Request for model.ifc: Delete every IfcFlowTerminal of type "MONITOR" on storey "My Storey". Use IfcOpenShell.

First a look at what the model holds.

```python
import ifcopenshell
import ifcopenshell.util.element

model = ifcopenshell.open("model.ifc")
print(model.schema)
storey = next(s for s in model.by_type("IfcBuildingStorey") if s.Name == "My Storey")
terminals = [e for e in ifcopenshell.util.element.get_decomposition(storey) if e.is_a("IfcFlowTerminal")]
seen = {}
for e in terminals:
    element_type = ifcopenshell.util.element.get_type(e)
    name = element_type.Name if element_type not in (None, e) else None
    seen[name] = seen.get(name, 0) + 1
for name, count in sorted(seen.items(), key=str):
    print(count, "x", name)
```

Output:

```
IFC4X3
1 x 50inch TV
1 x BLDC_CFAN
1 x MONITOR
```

```python
import ifcopenshell
import ifcopenshell.api.root
import ifcopenshell.util.element

model = ifcopenshell.open("model.ifc")

storey = next(s for s in model.by_type("IfcBuildingStorey") if s.Name == "My Storey")
terminals = [e for e in ifcopenshell.util.element.get_decomposition(storey) if e.is_a("IfcFlowTerminal")]
targets = [e for e in terminals if (t := ifcopenshell.util.element.get_type(e)) not in (None, e) and t.Name == "MONITOR"]

for e in targets:
    ifcopenshell.api.root.remove_product(model, product=e)
print(len(targets), "removed")

model.write("model-out.ifc")
```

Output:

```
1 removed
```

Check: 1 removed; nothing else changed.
